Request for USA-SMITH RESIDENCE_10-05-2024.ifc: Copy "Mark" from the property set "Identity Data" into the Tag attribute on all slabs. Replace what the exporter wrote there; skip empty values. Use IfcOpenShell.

First a look at what the model holds.

```python
import ifcopenshell
import ifcopenshell.util.element

model = ifcopenshell.open("USA-SMITH RESIDENCE_10-05-2024.ifc")
print(model.schema)
slabs = model.by_type("IfcSlab")
print(len(slabs), "slabs")
for e in slabs[:8]:
    source = ifcopenshell.util.element.get_pset(e, "Identity Data", "Mark")
    target = e.Tag
    print(e.id(), repr(source), repr(target), sep=" | ")
```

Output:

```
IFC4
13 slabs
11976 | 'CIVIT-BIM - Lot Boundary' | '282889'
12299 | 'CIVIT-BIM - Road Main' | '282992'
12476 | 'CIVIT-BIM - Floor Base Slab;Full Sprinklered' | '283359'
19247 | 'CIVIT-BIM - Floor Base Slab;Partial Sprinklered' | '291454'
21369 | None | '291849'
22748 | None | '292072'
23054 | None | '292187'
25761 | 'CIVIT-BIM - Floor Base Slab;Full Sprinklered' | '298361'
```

```python
import ifcopenshell
import ifcopenshell.util.element

model = ifcopenshell.open("USA-SMITH RESIDENCE_10-05-2024.ifc")

count = 0
for e in model.by_type("IfcSlab"):
    value = ifcopenshell.util.element.get_pset(e, "Identity Data", "Mark")
    current = e.Tag
    if not value or not value.strip() or current == value:
        continue
    e.Tag = value
    count += 1

print(count, "slabs updated")

model.write("USA-SMITH RESIDENCE_10-05-2024_edited.ifc")
```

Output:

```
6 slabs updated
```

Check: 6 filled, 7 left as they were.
